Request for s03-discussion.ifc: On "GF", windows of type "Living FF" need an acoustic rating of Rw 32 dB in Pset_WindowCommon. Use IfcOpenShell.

First a look at what the model holds.

```python
import ifcopenshell
import ifcopenshell.util.element

model = ifcopenshell.open("s03-discussion.ifc")
print(model.schema)
storey = next(s for s in model.by_type("IfcBuildingStorey") if s.Name == "GF")
windows = [e for e in ifcopenshell.util.element.get_decomposition(storey) if e.is_a("IfcWindow")]
seen = {}
for e in windows:
    element_type = ifcopenshell.util.element.get_type(e)
    key = (element_type.Name if element_type != e and element_type else None, ifcopenshell.util.element.get_pset(e, "Pset_WindowCommon", "AcousticRating"))
    seen[key] = seen.get(key, 0) + 1
for (name, value), count in sorted(seen.items(), key=str):
    print(count, "x", name, "|", value)
```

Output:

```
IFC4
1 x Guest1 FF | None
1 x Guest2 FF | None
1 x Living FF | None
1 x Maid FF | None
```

```python
import ifcopenshell
import ifcopenshell.api.pset
import ifcopenshell.util.element

model = ifcopenshell.open("s03-discussion.ifc")

storey = next(s for s in model.by_type("IfcBuildingStorey") if s.Name == "GF")
windows = [e for e in ifcopenshell.util.element.get_decomposition(storey) if e.is_a("IfcWindow")]

count = 0
for e in windows:
    element_type = ifcopenshell.util.element.get_type(e)
    if element_type in (None, e) or element_type.Name != "Living FF":
        continue
    # add_pset returns the element's existing set when there is one.
    pset = ifcopenshell.api.pset.add_pset(model, product=e, name="Pset_WindowCommon")
    ifcopenshell.api.pset.edit_pset(model, pset=pset, properties={"AcousticRating": "Rw 32 dB"})
    count += 1

print(count, "windows updated")

model.write("s03-discussion-out.ifc")
```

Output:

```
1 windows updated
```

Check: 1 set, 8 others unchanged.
